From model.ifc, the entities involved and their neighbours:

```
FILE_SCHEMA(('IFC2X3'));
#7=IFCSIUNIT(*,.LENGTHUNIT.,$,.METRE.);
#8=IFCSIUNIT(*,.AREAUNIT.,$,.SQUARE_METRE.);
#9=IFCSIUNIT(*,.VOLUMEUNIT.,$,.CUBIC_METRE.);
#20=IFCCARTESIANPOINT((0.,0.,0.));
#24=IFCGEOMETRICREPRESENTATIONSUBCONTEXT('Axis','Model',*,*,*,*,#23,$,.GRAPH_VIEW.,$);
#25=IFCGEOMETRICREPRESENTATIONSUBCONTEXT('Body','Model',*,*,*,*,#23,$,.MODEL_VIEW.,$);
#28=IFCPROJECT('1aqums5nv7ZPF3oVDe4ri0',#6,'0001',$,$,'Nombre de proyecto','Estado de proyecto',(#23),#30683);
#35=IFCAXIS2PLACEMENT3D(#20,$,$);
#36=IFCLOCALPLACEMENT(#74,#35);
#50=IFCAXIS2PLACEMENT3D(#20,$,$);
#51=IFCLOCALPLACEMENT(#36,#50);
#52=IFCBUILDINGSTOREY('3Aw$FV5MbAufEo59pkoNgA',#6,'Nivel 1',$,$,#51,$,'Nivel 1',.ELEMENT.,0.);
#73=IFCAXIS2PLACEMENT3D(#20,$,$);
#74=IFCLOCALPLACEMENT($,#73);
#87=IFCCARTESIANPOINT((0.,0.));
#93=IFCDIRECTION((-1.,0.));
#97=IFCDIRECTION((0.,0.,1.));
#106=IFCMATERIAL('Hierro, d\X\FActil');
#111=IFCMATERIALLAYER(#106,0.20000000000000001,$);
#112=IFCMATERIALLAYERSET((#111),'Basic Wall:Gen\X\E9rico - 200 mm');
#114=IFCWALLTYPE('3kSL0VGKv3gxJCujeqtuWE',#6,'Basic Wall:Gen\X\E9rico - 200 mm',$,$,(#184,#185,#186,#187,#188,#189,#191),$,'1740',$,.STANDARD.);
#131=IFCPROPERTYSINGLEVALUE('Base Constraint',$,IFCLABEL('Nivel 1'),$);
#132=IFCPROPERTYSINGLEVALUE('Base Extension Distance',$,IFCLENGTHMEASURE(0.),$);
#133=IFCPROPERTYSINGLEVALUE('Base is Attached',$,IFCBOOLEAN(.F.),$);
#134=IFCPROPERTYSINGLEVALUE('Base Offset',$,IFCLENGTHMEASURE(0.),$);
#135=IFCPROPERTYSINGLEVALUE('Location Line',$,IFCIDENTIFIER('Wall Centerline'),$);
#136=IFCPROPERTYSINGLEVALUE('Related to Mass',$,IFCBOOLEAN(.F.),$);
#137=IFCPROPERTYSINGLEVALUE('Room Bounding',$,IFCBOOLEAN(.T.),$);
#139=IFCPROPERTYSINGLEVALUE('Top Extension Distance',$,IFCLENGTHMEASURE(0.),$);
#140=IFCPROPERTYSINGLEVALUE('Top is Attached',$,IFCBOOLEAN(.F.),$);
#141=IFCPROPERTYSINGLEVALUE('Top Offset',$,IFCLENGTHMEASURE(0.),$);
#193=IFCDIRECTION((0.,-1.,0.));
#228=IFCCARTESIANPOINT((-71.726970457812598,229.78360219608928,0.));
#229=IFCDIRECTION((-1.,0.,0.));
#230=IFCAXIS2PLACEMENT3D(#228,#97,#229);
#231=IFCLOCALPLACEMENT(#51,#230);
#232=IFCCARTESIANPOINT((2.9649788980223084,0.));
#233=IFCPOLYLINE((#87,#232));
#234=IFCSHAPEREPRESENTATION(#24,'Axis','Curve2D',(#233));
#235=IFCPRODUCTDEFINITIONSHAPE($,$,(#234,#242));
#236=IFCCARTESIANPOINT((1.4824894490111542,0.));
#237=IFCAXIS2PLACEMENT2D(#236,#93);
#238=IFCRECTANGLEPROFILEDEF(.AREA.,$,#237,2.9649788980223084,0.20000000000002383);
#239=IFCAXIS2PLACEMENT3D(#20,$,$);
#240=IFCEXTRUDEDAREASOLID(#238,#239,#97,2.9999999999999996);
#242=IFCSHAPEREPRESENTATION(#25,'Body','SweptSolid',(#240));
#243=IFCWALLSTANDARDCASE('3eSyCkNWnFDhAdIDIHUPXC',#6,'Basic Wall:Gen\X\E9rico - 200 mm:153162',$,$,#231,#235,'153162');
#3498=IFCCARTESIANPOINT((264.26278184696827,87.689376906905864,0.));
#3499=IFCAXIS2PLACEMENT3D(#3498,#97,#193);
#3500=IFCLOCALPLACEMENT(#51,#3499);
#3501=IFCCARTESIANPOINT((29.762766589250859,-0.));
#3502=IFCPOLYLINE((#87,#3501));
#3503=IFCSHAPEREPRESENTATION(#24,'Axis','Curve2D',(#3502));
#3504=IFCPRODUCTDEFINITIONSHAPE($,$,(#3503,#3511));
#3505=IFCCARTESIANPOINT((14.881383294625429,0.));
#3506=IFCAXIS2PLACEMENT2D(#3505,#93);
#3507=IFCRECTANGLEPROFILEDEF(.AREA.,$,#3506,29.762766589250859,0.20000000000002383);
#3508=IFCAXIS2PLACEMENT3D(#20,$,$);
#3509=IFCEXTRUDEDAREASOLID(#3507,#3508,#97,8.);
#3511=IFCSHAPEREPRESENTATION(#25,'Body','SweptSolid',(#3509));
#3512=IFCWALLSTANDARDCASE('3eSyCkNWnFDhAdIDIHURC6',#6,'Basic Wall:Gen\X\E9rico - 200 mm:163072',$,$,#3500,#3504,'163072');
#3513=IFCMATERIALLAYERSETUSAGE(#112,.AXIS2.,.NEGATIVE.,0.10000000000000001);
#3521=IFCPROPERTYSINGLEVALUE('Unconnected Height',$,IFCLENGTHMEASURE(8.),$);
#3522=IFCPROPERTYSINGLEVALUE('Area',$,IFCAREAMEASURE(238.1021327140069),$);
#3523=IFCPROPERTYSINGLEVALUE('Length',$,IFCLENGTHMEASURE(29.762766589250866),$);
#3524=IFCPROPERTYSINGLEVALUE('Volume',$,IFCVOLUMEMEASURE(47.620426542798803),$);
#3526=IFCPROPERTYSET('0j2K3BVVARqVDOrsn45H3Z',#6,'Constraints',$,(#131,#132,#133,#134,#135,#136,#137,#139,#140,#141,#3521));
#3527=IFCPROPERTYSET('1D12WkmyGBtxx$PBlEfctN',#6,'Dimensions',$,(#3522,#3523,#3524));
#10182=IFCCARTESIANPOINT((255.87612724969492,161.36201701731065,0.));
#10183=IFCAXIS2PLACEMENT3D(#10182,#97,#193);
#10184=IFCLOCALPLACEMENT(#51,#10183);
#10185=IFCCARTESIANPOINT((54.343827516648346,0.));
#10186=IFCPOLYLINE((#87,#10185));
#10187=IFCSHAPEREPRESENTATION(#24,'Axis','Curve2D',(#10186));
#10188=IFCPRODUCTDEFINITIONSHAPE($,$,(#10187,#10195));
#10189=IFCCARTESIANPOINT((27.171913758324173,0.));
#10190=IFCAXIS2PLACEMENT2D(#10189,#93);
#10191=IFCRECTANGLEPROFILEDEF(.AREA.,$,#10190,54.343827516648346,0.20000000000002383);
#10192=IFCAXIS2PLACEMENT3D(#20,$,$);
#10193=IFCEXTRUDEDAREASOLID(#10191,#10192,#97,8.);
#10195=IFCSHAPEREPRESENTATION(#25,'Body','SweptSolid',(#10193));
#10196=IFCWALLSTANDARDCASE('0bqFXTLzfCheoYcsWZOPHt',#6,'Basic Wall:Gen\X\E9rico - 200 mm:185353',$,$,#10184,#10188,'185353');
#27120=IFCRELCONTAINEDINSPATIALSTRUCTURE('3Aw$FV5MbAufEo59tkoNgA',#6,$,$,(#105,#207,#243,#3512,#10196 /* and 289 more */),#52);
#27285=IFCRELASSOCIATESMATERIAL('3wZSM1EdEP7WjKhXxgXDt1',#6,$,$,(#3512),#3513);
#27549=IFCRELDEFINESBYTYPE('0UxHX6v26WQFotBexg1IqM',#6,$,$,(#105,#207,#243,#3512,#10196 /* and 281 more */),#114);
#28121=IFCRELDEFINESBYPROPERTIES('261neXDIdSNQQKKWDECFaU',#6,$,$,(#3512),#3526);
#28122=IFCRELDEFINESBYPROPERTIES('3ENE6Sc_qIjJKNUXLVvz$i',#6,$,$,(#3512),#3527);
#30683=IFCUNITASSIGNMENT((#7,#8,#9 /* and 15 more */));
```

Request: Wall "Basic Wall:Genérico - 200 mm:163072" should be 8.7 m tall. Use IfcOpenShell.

```python
import ifcopenshell
import ifcopenshell.api.pset
import ifcopenshell.geom
import ifcopenshell.util.element
import ifcopenshell.util.representation
import ifcopenshell.util.shape
import ifcopenshell.util.unit

model = ifcopenshell.open("model.ifc")
unit_scale = ifcopenshell.util.unit.calculate_unit_scale(model)
area_scale = ifcopenshell.util.unit.calculate_unit_scale(model, "AREAUNIT")
volume_scale = ifcopenshell.util.unit.calculate_unit_scale(model, "VOLUMEUNIT")
settings = ifcopenshell.geom.settings()


def volume(element):
    """Net volume in cubic metres, openings subtracted."""
    shape = ifcopenshell.geom.create_shape(settings, element)
    return ifcopenshell.util.shape.get_volume(shape.geometry)


wall = model.by_guid("3eSyCkNWnFDhAdIDIHURC6")
before = volume(wall)

body = ifcopenshell.util.representation.get_representation(wall, "Model", "Body")
solid = body.Items[0]
old_height = solid.Depth
solid.Depth = 8.7 / unit_scale
after = volume(wall)
thickness = 0.2  # wall thickness in metres

# Update the stored height, areas and volumes.
pset = model.by_id(ifcopenshell.util.element.get_pset(wall, "Constraints", should_inherit=False)["id"])
ifcopenshell.api.pset.edit_pset(model, pset=pset, properties={
    "Unconnected Height": model.create_entity("IfcLengthMeasure", solid.Depth),
})
pset = model.by_id(ifcopenshell.util.element.get_pset(wall, "Dimensions", should_inherit=False)["id"])
ifcopenshell.api.pset.edit_pset(model, pset=pset, properties={
    "Area": model.create_entity("IfcAreaMeasure", after / thickness / area_scale),
    "Volume": model.create_entity("IfcVolumeMeasure", after / volume_scale),
})

print(f"height {old_height:g} -> {solid.Depth:g}, volume {before:.3f} -> {after:.3f} m3")

model.write("model_updated.ifc")
```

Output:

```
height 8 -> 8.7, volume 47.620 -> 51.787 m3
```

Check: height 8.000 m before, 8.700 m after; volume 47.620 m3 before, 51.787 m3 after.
